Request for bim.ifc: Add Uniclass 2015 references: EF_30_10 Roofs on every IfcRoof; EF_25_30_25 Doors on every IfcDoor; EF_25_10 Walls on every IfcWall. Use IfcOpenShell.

First a look at what the model holds.

```python
import ifcopenshell

model = ifcopenshell.open("bim.ifc")
print(model.schema)
print("classifications:", [c.Name for c in model.by_type("IfcClassification")])
for ifc_class in ("IfcDoor", "IfcRoof", "IfcStair", "IfcWall", "IfcWindow"):
    print(ifc_class, len(model.by_type(ifc_class)))
```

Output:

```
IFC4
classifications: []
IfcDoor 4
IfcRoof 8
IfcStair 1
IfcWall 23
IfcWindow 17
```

```python
import ifcopenshell
import ifcopenshell.api.classification

model = ifcopenshell.open("bim.ifc")

system = ifcopenshell.api.classification.add_classification(model, classification="Uniclass 2015")

codes = {
    "IfcRoof": ("EF_30_10", "Roofs"),
    "IfcDoor": ("EF_25_30_25", "Doors"),
    "IfcWall": ("EF_25_10", "Walls"),
}
for ifc_class, (code, name) in codes.items():
    products = model.by_type(ifc_class)
    ifcopenshell.api.classification.add_reference(
        model, products=products, classification=system, identification=code, name=name
    )
    print(code, len(products))

model.write("bim_updated.ifc")
```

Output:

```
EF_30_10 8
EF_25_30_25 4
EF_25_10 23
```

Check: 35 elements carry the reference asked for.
